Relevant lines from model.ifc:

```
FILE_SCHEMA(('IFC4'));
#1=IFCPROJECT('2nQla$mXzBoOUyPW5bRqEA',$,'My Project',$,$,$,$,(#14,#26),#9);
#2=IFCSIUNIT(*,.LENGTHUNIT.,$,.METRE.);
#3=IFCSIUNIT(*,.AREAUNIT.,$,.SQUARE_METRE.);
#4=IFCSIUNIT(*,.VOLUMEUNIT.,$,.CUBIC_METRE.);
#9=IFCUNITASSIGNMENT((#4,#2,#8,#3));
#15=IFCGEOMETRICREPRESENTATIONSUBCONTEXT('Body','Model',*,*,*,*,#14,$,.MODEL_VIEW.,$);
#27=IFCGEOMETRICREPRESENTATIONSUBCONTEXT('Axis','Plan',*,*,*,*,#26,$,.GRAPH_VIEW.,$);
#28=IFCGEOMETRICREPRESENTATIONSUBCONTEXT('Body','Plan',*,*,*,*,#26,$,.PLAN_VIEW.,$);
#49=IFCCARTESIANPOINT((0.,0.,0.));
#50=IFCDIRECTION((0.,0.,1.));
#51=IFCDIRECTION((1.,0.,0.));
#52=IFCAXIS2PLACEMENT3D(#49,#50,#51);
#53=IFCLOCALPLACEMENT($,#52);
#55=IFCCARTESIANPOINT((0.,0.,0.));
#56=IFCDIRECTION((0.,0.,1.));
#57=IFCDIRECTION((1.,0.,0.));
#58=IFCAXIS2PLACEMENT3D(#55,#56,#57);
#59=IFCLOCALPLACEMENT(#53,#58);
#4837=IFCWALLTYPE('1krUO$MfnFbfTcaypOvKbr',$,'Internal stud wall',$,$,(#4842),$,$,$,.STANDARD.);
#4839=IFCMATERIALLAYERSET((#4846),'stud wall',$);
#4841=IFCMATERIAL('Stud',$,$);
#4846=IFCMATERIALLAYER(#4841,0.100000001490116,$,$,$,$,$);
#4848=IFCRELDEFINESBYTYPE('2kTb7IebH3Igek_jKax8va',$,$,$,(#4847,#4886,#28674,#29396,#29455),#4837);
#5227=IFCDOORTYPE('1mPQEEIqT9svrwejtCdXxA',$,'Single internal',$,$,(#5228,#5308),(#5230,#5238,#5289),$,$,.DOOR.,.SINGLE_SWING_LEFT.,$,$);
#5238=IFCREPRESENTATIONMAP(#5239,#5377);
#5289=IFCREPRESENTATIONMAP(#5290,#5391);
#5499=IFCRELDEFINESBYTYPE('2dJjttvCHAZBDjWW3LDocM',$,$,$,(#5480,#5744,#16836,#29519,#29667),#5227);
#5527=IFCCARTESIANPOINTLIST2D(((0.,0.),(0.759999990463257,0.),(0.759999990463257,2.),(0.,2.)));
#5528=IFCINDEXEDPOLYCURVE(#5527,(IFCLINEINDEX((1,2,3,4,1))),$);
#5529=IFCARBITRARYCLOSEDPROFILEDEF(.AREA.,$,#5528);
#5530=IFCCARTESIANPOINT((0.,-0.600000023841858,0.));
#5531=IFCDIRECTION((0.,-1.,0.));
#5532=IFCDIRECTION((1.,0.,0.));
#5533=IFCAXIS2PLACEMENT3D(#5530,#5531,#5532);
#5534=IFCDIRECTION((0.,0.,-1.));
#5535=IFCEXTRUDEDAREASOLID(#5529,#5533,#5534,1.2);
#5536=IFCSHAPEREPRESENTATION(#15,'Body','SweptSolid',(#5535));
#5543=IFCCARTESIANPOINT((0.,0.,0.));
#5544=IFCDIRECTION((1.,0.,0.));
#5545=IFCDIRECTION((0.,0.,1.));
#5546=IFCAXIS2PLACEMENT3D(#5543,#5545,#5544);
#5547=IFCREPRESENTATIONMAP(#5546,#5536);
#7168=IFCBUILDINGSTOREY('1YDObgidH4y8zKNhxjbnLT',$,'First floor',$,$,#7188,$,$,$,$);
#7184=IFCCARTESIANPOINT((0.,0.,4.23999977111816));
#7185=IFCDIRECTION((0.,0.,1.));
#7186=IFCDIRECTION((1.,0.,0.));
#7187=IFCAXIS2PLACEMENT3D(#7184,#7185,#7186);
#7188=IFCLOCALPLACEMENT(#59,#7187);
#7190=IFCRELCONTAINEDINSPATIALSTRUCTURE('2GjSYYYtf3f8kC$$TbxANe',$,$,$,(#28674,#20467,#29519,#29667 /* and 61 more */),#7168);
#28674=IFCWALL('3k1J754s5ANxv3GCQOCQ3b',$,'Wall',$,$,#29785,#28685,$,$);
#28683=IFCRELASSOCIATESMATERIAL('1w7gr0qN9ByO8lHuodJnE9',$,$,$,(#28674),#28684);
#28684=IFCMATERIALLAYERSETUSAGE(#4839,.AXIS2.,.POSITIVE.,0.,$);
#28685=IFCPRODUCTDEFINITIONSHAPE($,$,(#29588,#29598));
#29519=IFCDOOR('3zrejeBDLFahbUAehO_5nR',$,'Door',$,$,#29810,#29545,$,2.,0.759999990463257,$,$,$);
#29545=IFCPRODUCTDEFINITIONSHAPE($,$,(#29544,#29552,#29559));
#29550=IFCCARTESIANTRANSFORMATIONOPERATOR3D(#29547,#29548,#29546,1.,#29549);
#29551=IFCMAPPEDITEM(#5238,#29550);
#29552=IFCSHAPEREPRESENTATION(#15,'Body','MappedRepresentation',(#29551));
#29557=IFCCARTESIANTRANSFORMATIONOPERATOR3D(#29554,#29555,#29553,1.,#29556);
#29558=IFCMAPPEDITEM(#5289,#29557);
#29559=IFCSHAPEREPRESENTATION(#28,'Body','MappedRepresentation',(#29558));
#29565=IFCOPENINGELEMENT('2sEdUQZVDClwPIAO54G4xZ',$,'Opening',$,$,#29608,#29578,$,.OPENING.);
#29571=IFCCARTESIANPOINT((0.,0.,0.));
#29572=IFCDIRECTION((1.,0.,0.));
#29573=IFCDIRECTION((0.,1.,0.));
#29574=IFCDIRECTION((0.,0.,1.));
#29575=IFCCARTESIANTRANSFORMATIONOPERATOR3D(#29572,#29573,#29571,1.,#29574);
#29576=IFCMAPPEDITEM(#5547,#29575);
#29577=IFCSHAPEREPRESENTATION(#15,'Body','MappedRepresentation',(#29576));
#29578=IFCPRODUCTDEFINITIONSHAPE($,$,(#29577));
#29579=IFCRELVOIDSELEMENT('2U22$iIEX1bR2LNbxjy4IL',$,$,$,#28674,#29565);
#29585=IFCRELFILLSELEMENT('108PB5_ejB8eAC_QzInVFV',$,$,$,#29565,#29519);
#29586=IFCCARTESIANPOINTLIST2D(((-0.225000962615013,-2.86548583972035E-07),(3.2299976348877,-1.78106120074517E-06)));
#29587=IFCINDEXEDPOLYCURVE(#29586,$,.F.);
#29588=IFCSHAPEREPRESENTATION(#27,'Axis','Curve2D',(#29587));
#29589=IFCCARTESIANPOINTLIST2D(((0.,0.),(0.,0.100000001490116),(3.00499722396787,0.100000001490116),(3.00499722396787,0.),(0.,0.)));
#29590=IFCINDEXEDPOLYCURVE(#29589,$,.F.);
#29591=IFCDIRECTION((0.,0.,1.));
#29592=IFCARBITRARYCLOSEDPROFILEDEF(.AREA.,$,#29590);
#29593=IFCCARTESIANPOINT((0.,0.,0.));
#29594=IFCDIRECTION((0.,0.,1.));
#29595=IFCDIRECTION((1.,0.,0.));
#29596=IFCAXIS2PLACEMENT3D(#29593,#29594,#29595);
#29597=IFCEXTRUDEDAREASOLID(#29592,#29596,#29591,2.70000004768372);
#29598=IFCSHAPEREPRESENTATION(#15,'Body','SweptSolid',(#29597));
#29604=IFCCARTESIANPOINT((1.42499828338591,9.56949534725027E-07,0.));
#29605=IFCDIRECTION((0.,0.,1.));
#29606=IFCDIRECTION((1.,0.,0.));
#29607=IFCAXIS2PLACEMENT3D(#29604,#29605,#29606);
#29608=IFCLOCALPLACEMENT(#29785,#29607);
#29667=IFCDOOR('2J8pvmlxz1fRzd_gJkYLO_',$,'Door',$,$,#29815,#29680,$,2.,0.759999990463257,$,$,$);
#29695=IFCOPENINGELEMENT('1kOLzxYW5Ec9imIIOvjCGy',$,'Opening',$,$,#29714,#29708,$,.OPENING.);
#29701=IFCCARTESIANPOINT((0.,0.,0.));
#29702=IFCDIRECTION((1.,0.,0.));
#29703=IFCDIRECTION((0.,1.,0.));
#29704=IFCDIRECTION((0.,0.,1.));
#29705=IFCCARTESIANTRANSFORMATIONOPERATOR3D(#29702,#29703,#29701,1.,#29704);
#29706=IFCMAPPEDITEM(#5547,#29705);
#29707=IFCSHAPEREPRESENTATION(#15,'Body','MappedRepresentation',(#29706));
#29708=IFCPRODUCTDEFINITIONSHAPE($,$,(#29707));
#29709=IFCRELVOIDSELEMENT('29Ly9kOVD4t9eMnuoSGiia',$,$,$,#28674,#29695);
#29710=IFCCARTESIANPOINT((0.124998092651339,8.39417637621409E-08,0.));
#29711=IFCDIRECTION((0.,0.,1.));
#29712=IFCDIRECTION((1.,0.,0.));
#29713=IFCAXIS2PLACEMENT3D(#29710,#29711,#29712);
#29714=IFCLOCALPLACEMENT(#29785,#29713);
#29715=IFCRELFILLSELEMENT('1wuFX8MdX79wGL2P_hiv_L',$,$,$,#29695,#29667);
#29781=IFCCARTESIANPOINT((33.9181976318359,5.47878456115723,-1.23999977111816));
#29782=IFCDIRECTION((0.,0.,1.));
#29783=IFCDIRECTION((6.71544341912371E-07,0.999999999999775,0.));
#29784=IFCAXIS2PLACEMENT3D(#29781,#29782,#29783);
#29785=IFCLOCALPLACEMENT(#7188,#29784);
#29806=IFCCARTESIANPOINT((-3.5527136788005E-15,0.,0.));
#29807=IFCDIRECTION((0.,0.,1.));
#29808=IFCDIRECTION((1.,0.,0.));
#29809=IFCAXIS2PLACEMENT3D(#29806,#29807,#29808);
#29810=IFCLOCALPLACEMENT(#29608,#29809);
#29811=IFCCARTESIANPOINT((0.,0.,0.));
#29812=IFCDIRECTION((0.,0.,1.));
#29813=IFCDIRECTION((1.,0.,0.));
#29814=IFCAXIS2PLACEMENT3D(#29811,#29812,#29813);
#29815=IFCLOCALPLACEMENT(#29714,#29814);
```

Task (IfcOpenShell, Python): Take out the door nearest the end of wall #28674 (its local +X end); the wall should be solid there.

```python
import ifcopenshell
import ifcopenshell.api.feature
import ifcopenshell.api.root
import ifcopenshell.geom
import ifcopenshell.util.shape

model = ifcopenshell.open("model.ifc")
settings = ifcopenshell.geom.settings()


def volume(element):
    """Net volume in cubic metres, openings subtracted."""
    shape = ifcopenshell.geom.create_shape(settings, element)
    return ifcopenshell.util.shape.get_volume(shape.geometry)


door = model.by_guid("3zrejeBDLFahbUAehO_5nR")
opening = door.FillsVoids[0].RelatingOpeningElement
wall = opening.VoidsElements[0].RelatingBuildingElement
before = volume(wall)

ifcopenshell.api.root.remove_product(model, product=door)
ifcopenshell.api.feature.remove_feature(model, feature=opening)

after = volume(wall)

print(f"wall volume {before:.3f} -> {after:.3f} m3")

model.write("model_updated.ifc")
```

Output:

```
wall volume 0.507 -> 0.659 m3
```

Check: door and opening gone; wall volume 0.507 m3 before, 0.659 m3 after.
